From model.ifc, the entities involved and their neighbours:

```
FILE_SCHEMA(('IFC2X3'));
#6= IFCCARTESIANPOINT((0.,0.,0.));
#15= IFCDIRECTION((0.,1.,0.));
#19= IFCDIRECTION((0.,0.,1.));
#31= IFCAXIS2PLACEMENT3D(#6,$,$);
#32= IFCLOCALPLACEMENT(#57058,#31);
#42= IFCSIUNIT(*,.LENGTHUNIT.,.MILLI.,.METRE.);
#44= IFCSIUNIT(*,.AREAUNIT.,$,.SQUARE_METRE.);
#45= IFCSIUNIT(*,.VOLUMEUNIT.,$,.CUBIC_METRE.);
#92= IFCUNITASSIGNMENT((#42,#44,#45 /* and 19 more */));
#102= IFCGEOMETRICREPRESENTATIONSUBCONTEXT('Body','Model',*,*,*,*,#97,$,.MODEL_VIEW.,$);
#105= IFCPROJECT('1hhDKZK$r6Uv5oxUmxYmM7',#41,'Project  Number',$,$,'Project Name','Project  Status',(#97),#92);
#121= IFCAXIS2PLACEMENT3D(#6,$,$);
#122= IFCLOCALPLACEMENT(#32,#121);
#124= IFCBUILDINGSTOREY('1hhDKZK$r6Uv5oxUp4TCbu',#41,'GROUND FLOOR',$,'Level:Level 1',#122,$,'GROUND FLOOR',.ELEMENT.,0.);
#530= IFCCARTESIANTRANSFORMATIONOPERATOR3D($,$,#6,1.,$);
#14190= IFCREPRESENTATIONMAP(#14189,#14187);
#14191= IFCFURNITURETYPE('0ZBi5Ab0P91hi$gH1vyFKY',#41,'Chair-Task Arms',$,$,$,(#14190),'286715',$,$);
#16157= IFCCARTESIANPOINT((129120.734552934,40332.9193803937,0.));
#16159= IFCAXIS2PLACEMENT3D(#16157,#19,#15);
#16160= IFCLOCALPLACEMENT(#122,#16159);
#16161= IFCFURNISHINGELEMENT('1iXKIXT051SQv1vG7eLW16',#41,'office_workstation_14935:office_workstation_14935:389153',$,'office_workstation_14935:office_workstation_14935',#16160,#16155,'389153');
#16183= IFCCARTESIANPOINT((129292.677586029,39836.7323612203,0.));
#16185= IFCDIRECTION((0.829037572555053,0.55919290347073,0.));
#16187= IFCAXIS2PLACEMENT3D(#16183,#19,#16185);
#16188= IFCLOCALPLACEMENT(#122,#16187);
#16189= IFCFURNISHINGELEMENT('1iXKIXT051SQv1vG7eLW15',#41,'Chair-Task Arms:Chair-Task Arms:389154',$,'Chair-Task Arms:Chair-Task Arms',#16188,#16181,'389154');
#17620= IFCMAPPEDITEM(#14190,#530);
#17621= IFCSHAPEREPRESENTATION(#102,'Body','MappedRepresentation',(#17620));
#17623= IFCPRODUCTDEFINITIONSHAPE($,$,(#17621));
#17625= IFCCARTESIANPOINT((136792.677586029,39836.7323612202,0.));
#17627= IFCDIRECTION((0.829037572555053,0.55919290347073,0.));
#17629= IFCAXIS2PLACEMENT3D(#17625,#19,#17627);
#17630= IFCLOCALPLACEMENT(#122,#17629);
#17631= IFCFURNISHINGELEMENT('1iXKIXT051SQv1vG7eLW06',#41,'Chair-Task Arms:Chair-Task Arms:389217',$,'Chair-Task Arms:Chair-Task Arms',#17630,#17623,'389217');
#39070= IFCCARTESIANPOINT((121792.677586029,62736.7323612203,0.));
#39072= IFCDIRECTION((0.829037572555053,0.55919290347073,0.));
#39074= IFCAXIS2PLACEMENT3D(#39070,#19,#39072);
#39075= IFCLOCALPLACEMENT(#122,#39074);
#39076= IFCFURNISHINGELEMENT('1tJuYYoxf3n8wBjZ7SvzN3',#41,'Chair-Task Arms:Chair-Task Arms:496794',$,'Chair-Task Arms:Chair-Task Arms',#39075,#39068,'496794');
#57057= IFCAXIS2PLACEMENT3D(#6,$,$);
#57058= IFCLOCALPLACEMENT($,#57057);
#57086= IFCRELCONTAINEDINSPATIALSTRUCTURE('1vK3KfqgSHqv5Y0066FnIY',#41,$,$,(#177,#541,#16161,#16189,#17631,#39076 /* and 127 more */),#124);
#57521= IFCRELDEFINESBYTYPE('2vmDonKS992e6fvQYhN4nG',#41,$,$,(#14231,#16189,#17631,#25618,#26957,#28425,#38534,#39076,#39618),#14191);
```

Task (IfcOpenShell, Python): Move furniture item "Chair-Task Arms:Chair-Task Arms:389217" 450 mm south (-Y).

```python
import ifcopenshell
import ifcopenshell.api.geometry
import ifcopenshell.util.placement

model = ifcopenshell.open("model.ifc")

item = model.by_id(17631)
matrix = ifcopenshell.util.placement.get_local_placement(item.ObjectPlacement)
matrix[1, 3] -= 450.0
ifcopenshell.api.geometry.edit_object_placement(model, product=item, matrix=matrix, is_si=False)

print(ifcopenshell.util.placement.get_local_placement(item.ObjectPlacement).round(3) + 0.0)

model.write("model_updated.ifc")
```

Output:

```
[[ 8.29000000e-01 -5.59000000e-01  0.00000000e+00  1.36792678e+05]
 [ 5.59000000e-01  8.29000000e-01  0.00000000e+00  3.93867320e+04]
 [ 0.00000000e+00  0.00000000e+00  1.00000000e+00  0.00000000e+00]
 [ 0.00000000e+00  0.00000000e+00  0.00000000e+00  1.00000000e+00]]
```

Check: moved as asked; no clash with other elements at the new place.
